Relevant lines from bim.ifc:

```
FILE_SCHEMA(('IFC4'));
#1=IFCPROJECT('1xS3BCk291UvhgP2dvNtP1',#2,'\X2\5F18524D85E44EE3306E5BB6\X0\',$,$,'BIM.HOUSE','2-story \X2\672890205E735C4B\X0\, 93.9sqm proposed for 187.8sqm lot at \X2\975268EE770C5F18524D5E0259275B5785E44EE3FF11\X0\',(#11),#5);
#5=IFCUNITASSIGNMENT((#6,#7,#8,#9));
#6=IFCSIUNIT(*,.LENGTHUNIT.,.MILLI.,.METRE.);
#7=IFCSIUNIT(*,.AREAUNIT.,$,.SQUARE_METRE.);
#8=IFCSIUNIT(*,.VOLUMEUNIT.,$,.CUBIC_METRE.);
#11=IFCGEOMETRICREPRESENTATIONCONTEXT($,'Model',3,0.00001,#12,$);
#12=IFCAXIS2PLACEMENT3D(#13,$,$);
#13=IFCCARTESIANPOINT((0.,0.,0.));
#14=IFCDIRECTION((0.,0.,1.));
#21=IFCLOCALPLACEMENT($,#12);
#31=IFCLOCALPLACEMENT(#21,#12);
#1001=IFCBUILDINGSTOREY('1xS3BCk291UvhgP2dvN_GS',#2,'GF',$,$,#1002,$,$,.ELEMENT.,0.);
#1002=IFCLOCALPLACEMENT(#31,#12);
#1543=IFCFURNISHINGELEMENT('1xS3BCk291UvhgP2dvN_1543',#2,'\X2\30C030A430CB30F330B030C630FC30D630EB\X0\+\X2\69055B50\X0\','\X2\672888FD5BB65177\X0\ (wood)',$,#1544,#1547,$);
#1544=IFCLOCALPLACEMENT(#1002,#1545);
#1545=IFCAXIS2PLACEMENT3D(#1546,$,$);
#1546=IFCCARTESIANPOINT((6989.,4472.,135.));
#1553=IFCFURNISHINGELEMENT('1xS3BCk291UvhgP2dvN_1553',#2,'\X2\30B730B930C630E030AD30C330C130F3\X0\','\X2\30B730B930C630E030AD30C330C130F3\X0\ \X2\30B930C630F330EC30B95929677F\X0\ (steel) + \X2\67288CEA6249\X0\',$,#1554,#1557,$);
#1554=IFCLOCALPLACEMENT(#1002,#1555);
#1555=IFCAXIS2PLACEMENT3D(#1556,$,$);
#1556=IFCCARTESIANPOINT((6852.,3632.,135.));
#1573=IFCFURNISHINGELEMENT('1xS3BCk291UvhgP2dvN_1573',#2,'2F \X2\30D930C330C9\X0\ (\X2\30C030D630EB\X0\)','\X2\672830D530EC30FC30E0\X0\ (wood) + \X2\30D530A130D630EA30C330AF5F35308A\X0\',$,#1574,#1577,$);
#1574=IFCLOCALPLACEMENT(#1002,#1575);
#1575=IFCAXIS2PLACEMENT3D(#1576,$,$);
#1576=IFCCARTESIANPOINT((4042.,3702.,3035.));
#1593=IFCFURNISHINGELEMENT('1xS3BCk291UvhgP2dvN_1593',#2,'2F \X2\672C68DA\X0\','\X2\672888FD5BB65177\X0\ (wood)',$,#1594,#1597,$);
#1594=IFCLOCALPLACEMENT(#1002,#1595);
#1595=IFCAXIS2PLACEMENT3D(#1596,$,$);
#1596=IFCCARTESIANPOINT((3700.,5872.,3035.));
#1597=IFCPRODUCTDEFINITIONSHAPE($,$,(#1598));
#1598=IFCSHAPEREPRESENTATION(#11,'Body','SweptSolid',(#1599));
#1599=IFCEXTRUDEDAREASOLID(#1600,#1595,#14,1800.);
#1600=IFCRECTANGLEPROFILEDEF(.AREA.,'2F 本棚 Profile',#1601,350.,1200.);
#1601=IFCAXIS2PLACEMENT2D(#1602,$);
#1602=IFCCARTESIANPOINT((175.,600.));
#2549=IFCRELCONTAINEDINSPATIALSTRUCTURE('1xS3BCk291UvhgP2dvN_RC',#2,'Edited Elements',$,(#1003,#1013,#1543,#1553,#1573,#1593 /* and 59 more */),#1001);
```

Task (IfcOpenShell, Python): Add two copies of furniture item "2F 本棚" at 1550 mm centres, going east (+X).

```python
import numpy as np
import ifcopenshell
import ifcopenshell.api.geometry
import ifcopenshell.api.root
import ifcopenshell.util.element
import ifcopenshell.util.placement
import ifcopenshell.util.unit

model = ifcopenshell.open("bim.ifc")
unit_scale = ifcopenshell.util.unit.calculate_unit_scale(model)


def reuse_history(source, copy):
    """copy_class also copies each property set's owner history, people and application; keep the originals."""
    for rel in copy.IsDefinedBy:
        if rel.is_a("IfcRelDefinesByProperties") and (history := rel.RelatingPropertyDefinition.OwnerHistory):
            rel.RelatingPropertyDefinition.OwnerHistory = source.OwnerHistory
            ifcopenshell.util.element.remove_deep2(model, history)


source = model.by_guid("1xS3BCk291UvhgP2dvN_1593")
base = ifcopenshell.util.placement.get_local_placement(source.ObjectPlacement)
step = np.array([1.0, 0.0, 0.0]) * 1.55 / unit_scale

for i in range(1, 3):
    copy = ifcopenshell.api.root.copy_class(model, product=source)
    copy.Representation = ifcopenshell.util.element.copy_deep(
        model, source.Representation, exclude=["IfcGeometricRepresentationContext", "IfcRepresentationMap"]
    )
    reuse_history(source, copy)
    matrix = base.copy()
    matrix[:3, 3] += i * step
    print("added at", matrix[:3, 3].round(3) + 0.0)
    ifcopenshell.api.geometry.edit_object_placement(model, product=copy, matrix=matrix, is_si=False)

model.write("bim-out.ifc")
```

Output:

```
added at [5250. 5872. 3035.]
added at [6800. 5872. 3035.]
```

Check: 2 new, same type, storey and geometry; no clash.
